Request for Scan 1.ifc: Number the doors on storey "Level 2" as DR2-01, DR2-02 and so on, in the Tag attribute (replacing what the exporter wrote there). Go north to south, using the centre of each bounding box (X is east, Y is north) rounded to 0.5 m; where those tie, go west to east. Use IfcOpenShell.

First a look at what the model holds.

```python
import ifcopenshell
import ifcopenshell.util.element
import ifcopenshell.util.placement

model = ifcopenshell.open("Scan 1.ifc")
print(model.schema)
storey = next(s for s in model.by_type("IfcBuildingStorey") if s.Name == "Level 2")
doors = [e for e in ifcopenshell.util.element.get_decomposition(storey) if e.is_a("IfcDoor")]
for e in sorted(doors, key=lambda e: e.id()):
    origin = ifcopenshell.util.placement.get_local_placement(e.ObjectPlacement)[:3, 3]
    print(e.id(), e.Tag, e.Name, origin.round(2) + 0.0, sep=" | ")
```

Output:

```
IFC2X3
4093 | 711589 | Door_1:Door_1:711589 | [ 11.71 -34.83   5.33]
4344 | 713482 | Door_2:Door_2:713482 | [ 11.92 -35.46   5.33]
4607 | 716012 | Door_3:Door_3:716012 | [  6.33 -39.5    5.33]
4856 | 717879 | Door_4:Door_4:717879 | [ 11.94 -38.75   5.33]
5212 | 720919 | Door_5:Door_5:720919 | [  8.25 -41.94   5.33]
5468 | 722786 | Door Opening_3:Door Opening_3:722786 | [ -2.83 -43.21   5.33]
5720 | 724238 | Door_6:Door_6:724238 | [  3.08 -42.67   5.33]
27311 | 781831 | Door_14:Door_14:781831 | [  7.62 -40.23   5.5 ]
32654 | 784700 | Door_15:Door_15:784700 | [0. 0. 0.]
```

```python
import ifcopenshell
import ifcopenshell.geom
import ifcopenshell.util.element
import ifcopenshell.util.shape

model = ifcopenshell.open("Scan 1.ifc")
settings = ifcopenshell.geom.settings()
settings.set("use-world-coords", True)


def centre(element):
    shape = ifcopenshell.geom.create_shape(settings, element)
    return ifcopenshell.util.shape.get_bbox_centroid(shape.geometry)


storey = next(s for s in model.by_type("IfcBuildingStorey") if s.Name == "Level 2")
doors = [e for e in ifcopenshell.util.element.get_decomposition(storey) if e.is_a("IfcDoor")]

# Insertion points can sit at a corner or the storey origin, so sort by the geometry (in metres).
centres = {e: centre(e) for e in doors}
doors.sort(key=lambda e: (-round(centres[e][1] / 0.5), centres[e][0]))

for i, e in enumerate(doors, start=1):
    number = f"DR2-{i:02d}"
    e.Tag = number
    print(e.id(), number)

model.write("Scan 1_updated.ifc")
```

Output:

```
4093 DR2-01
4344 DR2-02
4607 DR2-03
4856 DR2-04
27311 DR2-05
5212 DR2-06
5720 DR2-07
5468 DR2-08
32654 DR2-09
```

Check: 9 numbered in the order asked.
